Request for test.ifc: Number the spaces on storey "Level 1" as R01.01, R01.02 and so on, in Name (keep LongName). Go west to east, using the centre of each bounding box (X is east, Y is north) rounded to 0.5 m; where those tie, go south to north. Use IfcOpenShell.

First a look at what the model holds.

```python
import ifcopenshell
import ifcopenshell.util.element
import ifcopenshell.util.placement

model = ifcopenshell.open("test.ifc")
print(model.schema)
storey = next(s for s in model.by_type("IfcBuildingStorey") if s.Name == "Level 1")
spaces = [e for e in ifcopenshell.util.element.get_decomposition(storey) if e.is_a("IfcSpace")]
for e in sorted(spaces, key=lambda e: e.id()):
    origin = ifcopenshell.util.placement.get_local_placement(e.ObjectPlacement)[:3, 3]
    print(e.id(), e.Name, e.LongName, origin.round(2) + 0.0, sep=" | ")
```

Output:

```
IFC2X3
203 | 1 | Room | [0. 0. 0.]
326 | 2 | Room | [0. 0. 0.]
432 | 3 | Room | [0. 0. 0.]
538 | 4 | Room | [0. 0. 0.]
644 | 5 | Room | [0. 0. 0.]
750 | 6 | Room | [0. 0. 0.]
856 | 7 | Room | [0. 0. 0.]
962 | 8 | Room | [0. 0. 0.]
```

```python
import ifcopenshell
import ifcopenshell.geom
import ifcopenshell.util.element
import ifcopenshell.util.shape

model = ifcopenshell.open("test.ifc")
settings = ifcopenshell.geom.settings()
settings.set("use-world-coords", True)


def centre(element):
    shape = ifcopenshell.geom.create_shape(settings, element)
    return ifcopenshell.util.shape.get_bbox_centroid(shape.geometry)


storey = next(s for s in model.by_type("IfcBuildingStorey") if s.Name == "Level 1")
spaces = [e for e in ifcopenshell.util.element.get_decomposition(storey) if e.is_a("IfcSpace")]

# Insertion points can sit at a corner or the storey origin, so sort by the geometry (in metres).
centres = {e: centre(e) for e in spaces}
spaces.sort(key=lambda e: (round(centres[e][0] / 0.5), centres[e][1]))

for i, e in enumerate(spaces, start=1):
    number = f"R01.{i:02d}"
    e.Name = number
    print(e.id(), number)

model.write("test_v2.ifc")
```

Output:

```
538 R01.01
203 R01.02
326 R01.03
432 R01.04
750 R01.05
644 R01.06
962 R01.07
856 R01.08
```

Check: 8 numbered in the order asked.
